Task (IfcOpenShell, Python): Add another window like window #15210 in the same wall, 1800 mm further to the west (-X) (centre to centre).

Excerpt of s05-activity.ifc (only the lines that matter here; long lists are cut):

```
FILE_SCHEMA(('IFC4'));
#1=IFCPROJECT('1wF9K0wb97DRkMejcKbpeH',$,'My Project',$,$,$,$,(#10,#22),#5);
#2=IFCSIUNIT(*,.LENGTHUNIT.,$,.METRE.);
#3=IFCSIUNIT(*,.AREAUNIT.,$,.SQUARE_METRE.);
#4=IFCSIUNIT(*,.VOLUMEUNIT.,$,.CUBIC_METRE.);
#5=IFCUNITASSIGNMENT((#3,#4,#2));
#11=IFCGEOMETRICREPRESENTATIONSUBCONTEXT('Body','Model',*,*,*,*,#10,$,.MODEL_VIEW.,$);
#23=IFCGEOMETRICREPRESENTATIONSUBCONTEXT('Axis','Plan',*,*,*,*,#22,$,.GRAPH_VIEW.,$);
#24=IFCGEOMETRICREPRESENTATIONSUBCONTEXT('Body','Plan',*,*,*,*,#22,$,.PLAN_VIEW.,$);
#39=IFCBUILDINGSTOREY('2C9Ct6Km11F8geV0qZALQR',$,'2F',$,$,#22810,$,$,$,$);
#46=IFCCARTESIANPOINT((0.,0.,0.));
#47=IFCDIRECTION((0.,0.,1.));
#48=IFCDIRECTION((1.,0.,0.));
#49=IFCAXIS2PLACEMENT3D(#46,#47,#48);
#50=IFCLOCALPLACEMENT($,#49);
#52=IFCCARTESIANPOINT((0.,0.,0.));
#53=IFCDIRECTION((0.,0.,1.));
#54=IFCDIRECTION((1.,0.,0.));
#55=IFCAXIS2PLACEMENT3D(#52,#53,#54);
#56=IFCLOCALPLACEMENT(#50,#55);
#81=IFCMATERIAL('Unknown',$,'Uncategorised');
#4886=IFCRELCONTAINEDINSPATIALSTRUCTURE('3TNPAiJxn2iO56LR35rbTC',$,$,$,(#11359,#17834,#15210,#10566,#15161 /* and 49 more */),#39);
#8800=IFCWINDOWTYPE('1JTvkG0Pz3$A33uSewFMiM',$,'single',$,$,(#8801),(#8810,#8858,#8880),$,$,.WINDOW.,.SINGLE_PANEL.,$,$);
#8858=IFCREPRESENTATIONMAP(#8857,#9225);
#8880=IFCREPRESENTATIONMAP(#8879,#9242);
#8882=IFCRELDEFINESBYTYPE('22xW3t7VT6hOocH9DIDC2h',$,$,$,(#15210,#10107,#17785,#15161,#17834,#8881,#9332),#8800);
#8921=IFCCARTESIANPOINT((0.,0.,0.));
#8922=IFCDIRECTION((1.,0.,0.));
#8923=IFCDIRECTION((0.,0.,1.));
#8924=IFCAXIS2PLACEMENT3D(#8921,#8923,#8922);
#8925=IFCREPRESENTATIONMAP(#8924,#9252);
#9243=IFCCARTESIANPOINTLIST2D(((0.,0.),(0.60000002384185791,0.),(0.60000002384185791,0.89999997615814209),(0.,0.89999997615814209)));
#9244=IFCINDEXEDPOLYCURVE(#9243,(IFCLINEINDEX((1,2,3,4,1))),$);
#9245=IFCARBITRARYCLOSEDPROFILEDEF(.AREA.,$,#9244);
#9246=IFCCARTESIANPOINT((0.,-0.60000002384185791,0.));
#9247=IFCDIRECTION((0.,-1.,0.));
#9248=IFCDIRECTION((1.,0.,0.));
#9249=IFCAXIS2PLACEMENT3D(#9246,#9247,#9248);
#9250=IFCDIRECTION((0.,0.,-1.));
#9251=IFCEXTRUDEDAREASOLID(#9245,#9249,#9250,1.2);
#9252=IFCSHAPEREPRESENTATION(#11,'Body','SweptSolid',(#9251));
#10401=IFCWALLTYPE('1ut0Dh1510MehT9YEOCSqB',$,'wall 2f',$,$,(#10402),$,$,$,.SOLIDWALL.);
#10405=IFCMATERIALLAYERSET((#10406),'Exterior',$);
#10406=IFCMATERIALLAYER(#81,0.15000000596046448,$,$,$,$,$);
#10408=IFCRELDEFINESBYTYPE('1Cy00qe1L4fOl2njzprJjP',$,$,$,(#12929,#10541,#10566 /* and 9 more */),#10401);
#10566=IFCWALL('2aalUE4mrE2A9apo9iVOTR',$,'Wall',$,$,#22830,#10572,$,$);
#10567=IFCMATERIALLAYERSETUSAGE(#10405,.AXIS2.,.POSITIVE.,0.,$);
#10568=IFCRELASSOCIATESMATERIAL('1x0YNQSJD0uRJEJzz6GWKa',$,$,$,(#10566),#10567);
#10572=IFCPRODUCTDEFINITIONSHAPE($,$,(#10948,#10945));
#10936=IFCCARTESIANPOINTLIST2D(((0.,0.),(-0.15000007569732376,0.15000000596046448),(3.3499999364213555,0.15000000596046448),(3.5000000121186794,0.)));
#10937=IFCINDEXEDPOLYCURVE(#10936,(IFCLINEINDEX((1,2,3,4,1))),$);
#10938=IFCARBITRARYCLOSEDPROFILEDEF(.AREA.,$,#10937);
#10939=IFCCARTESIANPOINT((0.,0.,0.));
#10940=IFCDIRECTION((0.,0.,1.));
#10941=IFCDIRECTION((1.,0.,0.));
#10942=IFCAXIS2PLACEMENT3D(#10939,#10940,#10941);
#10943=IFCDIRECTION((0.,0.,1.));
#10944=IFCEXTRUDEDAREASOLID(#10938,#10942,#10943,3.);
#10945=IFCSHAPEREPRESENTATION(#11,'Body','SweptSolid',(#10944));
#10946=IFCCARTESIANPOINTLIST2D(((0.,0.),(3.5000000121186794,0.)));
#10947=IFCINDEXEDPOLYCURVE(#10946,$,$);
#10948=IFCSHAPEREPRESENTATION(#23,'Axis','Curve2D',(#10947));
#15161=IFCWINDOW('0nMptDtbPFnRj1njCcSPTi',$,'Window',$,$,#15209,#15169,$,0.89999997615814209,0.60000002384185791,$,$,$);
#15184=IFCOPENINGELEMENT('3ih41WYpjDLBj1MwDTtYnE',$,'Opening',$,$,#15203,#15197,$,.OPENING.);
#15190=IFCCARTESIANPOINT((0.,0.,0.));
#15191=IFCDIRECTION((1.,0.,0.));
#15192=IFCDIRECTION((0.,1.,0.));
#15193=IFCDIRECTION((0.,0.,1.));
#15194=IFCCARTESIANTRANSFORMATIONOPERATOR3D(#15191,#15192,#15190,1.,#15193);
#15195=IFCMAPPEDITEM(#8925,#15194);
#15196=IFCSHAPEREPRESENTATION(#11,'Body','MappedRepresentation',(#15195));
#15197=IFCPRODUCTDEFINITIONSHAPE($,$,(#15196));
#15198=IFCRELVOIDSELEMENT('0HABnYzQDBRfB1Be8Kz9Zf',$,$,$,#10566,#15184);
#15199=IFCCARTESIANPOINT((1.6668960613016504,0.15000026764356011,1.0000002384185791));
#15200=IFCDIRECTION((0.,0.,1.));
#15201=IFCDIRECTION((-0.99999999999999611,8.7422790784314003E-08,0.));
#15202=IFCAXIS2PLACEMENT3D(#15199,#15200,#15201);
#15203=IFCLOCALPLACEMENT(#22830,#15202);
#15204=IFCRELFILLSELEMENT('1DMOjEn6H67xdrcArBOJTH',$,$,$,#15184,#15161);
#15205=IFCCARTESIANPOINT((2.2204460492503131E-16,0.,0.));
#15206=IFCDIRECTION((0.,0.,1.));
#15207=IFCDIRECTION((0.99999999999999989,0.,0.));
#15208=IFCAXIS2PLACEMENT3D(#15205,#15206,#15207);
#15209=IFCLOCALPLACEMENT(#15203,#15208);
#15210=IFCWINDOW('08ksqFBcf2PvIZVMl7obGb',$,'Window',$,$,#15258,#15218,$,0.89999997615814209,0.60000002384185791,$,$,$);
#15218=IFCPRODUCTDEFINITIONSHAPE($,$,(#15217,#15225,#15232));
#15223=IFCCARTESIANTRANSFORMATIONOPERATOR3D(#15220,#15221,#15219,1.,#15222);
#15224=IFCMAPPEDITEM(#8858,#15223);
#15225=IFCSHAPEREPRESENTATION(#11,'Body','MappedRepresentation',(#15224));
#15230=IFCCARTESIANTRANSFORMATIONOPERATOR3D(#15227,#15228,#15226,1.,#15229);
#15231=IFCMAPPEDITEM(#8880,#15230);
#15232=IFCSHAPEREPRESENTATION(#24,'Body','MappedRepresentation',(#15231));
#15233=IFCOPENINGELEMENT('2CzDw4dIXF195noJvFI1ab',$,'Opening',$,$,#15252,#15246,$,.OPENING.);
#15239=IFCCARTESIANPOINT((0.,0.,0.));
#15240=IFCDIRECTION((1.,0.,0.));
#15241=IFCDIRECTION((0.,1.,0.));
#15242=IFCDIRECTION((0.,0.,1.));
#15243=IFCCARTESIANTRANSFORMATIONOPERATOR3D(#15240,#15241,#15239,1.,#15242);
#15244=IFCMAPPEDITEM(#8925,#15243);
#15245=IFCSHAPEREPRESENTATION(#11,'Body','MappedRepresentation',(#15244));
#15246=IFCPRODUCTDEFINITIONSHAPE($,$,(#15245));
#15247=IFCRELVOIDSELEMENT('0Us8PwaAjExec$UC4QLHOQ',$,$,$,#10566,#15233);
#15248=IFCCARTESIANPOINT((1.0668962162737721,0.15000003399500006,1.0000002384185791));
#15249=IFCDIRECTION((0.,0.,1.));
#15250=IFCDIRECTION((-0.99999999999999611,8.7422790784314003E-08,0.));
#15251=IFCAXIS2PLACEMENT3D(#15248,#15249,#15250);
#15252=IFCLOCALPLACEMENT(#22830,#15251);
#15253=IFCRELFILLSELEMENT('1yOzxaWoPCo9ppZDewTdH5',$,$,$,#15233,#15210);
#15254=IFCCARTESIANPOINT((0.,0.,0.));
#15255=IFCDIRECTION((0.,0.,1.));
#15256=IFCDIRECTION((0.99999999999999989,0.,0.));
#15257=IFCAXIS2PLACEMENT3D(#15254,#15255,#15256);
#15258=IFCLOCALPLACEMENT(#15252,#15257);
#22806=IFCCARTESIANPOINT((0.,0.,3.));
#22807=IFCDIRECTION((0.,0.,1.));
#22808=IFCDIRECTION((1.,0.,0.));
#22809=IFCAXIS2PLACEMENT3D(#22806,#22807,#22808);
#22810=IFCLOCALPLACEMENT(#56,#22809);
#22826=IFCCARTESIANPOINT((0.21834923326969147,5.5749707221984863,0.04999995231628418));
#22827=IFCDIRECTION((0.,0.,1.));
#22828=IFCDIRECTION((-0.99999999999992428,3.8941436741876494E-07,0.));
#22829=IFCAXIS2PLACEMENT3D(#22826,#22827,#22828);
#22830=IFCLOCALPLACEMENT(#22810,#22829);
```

```python
import ifcopenshell
import ifcopenshell.api.feature
import ifcopenshell.api.geometry
import ifcopenshell.api.root
import ifcopenshell.geom
import ifcopenshell.util.element
import ifcopenshell.util.placement
import ifcopenshell.util.shape
import ifcopenshell.util.unit

model = ifcopenshell.open("s05-activity.ifc")
unit_scale = ifcopenshell.util.unit.calculate_unit_scale(model)
settings = ifcopenshell.geom.settings()


def volume(element):
    """Net volume in cubic metres, openings subtracted."""
    shape = ifcopenshell.geom.create_shape(settings, element)
    return ifcopenshell.util.shape.get_volume(shape.geometry)


window = model.by_guid("08ksqFBcf2PvIZVMl7obGb")
opening = window.FillsVoids[0].RelatingOpeningElement
wall = opening.VoidsElements[0].RelatingBuildingElement
before = volume(wall)
shift = ifcopenshell.util.placement.get_local_placement(wall.ObjectPlacement)[:3, 0] * 1.8 / unit_scale

# copy_class copies the void relationship, type, container and properties, but no geometry.
new_opening = ifcopenshell.api.root.copy_class(model, product=opening)
new_opening.Representation = ifcopenshell.util.element.copy_deep(
    model, opening.Representation, exclude=["IfcGeometricRepresentationContext", "IfcRepresentationMap"]
)
new_window = ifcopenshell.api.root.copy_class(model, product=window)
new_window.Representation = ifcopenshell.util.element.copy_deep(
    model, window.Representation, exclude=["IfcGeometricRepresentationContext", "IfcRepresentationMap"]
)
ifcopenshell.api.feature.add_filling(model, opening=new_opening, element=new_window)

for old, new in ((opening, new_opening), (window, new_window)):
    matrix = ifcopenshell.util.placement.get_local_placement(old.ObjectPlacement)
    matrix[:3, 3] += shift
    ifcopenshell.api.geometry.edit_object_placement(model, product=new, matrix=matrix, is_si=False)

after = volume(wall)

print(f"wall volume {before:.3f} -> {after:.3f} m3")

model.write("s05-activity_v2.ifc")
```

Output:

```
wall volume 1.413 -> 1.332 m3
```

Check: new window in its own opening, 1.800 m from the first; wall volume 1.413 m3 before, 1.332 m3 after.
